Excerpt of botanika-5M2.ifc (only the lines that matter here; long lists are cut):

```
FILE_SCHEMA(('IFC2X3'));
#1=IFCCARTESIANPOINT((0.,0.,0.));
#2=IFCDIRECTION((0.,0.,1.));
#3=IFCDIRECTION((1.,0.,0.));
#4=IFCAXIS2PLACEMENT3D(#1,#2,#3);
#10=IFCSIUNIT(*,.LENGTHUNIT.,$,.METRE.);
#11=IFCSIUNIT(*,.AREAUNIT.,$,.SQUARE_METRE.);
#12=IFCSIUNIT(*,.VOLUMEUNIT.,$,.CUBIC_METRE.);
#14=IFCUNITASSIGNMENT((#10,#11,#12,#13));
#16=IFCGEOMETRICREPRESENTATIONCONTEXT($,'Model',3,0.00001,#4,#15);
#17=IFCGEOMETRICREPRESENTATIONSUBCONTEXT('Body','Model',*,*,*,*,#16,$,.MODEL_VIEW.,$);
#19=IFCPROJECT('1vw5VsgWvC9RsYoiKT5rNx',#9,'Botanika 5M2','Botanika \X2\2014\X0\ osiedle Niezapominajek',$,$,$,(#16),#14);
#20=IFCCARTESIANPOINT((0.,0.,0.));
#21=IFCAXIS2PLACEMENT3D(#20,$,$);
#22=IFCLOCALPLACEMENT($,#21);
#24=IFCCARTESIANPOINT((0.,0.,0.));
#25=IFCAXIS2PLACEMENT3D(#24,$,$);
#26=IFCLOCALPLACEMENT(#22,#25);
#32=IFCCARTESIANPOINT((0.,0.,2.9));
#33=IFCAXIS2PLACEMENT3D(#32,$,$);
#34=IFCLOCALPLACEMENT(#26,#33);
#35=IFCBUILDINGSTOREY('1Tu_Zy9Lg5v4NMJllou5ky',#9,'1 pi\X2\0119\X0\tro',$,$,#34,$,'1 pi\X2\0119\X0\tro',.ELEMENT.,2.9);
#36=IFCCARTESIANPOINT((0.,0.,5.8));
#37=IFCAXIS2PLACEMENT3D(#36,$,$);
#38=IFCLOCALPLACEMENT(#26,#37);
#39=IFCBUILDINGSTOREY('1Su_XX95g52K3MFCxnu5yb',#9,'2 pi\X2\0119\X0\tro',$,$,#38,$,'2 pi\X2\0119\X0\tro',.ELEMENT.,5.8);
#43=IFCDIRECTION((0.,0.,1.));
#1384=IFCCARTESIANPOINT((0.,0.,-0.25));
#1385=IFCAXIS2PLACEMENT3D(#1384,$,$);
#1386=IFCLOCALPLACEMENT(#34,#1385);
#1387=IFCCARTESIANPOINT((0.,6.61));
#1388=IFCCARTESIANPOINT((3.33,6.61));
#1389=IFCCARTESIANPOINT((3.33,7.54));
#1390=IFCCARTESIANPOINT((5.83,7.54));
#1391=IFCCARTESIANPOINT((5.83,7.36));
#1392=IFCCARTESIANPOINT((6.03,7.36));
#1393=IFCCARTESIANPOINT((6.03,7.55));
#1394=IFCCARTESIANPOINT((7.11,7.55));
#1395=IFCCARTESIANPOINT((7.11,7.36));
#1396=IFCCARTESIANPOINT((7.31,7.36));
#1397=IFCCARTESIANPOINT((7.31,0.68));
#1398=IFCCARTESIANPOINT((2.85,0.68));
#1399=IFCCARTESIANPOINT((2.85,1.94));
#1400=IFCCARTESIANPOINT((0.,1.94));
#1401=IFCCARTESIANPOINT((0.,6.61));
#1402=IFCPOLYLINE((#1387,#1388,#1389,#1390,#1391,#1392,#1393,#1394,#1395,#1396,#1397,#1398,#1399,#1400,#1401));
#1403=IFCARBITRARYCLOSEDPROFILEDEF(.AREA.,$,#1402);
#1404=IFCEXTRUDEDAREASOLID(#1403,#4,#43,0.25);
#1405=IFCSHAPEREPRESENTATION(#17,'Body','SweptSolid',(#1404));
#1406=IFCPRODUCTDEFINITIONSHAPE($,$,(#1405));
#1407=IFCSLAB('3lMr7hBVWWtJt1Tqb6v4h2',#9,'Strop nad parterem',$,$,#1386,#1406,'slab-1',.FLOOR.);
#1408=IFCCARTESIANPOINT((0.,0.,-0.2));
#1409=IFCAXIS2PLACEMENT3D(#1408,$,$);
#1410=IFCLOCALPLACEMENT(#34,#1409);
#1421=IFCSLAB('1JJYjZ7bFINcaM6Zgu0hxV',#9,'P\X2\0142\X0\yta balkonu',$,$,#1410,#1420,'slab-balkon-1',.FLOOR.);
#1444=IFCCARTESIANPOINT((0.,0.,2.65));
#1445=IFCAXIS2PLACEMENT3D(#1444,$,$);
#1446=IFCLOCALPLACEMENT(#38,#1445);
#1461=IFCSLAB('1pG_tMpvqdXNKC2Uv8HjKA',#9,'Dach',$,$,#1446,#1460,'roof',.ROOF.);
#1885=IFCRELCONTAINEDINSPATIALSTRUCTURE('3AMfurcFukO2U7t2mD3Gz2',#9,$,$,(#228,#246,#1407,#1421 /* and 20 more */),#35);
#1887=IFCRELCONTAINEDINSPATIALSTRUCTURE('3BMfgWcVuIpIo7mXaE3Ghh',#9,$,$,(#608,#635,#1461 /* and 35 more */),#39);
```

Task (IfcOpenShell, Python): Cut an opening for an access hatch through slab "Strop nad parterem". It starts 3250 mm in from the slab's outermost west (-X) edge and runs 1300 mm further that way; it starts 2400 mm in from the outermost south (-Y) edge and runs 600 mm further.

```python
import numpy as np
import ifcopenshell
import ifcopenshell.api.feature
import ifcopenshell.api.geometry
import ifcopenshell.api.root
import ifcopenshell.geom
import ifcopenshell.util.placement
import ifcopenshell.util.representation
import ifcopenshell.util.shape
import ifcopenshell.util.unit

model = ifcopenshell.open("botanika-5M2.ifc")
unit_scale = ifcopenshell.util.unit.calculate_unit_scale(model)
settings = ifcopenshell.geom.settings()


def volume(element):
    """Net volume in cubic metres, openings subtracted."""
    shape = ifcopenshell.geom.create_shape(settings, element)
    return ifcopenshell.util.shape.get_volume(shape.geometry)


slab = model.by_id(1407)
before = volume(slab)

# Extent in the slab's own axes, in metres. The edges named are its -X and -Y sides.
slab_shape = ifcopenshell.geom.create_shape(settings, slab)
vertices = ifcopenshell.util.shape.get_vertices(slab_shape.geometry)
x_min, y_min, bottom = vertices.min(axis=0)
top = vertices[:, 2].max()

opening = ifcopenshell.api.root.create_entity(model, ifc_class="IfcOpeningElement", name="Access hatch opening")
context = ifcopenshell.util.representation.get_context(model, "Model", "Body", "MODEL_VIEW")
width, depth = 1.3, 0.6
outline = [(0.0, 0.0), (width, 0.0), (width, depth), (0.0, depth), (0.0, 0.0)]
# Overshoot both faces by 50 mm so the cut is clean.
shape = ifcopenshell.api.geometry.add_slab_representation(
    model, context=context, depth=top - bottom + 0.1, polyline=outline
)
ifcopenshell.api.geometry.assign_representation(model, product=opening, representation=shape)

matrix = ifcopenshell.util.placement.get_local_placement(slab.ObjectPlacement)
matrix[:, 3] = matrix @ np.append(np.array([x_min + 3.25, y_min + 2.4, bottom - 0.05]) / unit_scale, 1.0)
ifcopenshell.api.geometry.edit_object_placement(model, product=opening, matrix=matrix, is_si=False)
ifcopenshell.api.feature.add_feature(model, feature=opening, element=slab)

after = volume(slab)

print(f"slab volume {before:.3f} -> {after:.3f} m3")

model.write("botanika-5M2_rev.ifc")
```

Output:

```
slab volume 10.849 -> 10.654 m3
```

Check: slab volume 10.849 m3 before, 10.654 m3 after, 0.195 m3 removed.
